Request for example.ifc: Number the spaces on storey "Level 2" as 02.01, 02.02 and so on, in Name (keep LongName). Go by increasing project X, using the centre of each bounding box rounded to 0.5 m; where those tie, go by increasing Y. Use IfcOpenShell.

First a look at what the model holds.

```python
import ifcopenshell
import ifcopenshell.util.element
import ifcopenshell.util.placement

model = ifcopenshell.open("example.ifc")
print(model.schema)
storey = next(s for s in model.by_type("IfcBuildingStorey") if s.Name == "Level 2")
spaces = [e for e in ifcopenshell.util.element.get_decomposition(storey) if e.is_a("IfcSpace")]
for e in sorted(spaces, key=lambda e: e.id()):
    origin = ifcopenshell.util.placement.get_local_placement(e.ObjectPlacement)[:3, 3]
    print(e.id(), e.Name, e.LongName, origin.round(2) + 0.0, sep=" | ")
```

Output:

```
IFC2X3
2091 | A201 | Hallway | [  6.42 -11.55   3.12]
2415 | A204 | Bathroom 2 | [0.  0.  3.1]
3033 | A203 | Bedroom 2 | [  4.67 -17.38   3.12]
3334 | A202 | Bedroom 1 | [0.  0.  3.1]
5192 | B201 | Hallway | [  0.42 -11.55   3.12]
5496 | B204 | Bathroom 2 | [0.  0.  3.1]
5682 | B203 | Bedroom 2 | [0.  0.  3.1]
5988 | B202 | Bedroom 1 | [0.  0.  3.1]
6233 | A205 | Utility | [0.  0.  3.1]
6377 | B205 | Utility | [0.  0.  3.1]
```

```python
import ifcopenshell
import ifcopenshell.geom
import ifcopenshell.util.element
import ifcopenshell.util.shape

model = ifcopenshell.open("example.ifc")
settings = ifcopenshell.geom.settings()
settings.set("use-world-coords", True)


def centre(element):
    shape = ifcopenshell.geom.create_shape(settings, element)
    return ifcopenshell.util.shape.get_bbox_centroid(shape.geometry)


storey = next(s for s in model.by_type("IfcBuildingStorey") if s.Name == "Level 2")
spaces = [e for e in ifcopenshell.util.element.get_decomposition(storey) if e.is_a("IfcSpace")]

# Insertion points can sit at a corner or the storey origin, so sort by the geometry (in metres).
centres = {e: centre(e) for e in spaces}
spaces.sort(key=lambda e: (round(centres[e][0] / 0.5), centres[e][1]))

for i, e in enumerate(spaces, start=1):
    number = f"02.{i:02d}"
    e.Name = number
    print(e.id(), number)

model.write("example_edited.ifc")
```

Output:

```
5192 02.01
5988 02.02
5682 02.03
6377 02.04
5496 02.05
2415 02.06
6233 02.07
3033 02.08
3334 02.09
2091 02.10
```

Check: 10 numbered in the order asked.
